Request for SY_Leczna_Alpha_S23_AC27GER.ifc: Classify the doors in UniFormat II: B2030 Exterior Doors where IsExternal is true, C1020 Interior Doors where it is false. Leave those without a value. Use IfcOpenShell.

First a look at what the model holds.

```python
import ifcopenshell
import ifcopenshell.util.element

model = ifcopenshell.open("SY_Leczna_Alpha_S23_AC27GER.ifc")
print(model.schema)
print("classifications:", [c.Name for c in model.by_type("IfcClassification")])
values = [ifcopenshell.util.element.get_pset(e, "Pset_DoorCommon", "IsExternal") for e in model.by_type("IfcDoor")]
for value in (True, False, None):
    print("IsExternal", value, values.count(value))
```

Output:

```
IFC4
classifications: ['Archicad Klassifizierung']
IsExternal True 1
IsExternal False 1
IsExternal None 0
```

```python
import ifcopenshell
import ifcopenshell.api.classification
import ifcopenshell.util.element

model = ifcopenshell.open("SY_Leczna_Alpha_S23_AC27GER.ifc")

system = ifcopenshell.api.classification.add_classification(model, classification="UniFormat II")

doors = model.by_type("IfcDoor")
external = {e: ifcopenshell.util.element.get_pset(e, "Pset_DoorCommon", "IsExternal") for e in doors}
for flag, code, name in ((True, "B2030", "Exterior Doors"), (False, "C1020", "Interior Doors")):
    products = [e for e in doors if external[e] is flag]
    ifcopenshell.api.classification.add_reference(
        model, products=products, classification=system, identification=code, name=name
    )
    print(code, len(products))

model.write("SY_Leczna_Alpha_S23_AC27GER_v2.ifc")
```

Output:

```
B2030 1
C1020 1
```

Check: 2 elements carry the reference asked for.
